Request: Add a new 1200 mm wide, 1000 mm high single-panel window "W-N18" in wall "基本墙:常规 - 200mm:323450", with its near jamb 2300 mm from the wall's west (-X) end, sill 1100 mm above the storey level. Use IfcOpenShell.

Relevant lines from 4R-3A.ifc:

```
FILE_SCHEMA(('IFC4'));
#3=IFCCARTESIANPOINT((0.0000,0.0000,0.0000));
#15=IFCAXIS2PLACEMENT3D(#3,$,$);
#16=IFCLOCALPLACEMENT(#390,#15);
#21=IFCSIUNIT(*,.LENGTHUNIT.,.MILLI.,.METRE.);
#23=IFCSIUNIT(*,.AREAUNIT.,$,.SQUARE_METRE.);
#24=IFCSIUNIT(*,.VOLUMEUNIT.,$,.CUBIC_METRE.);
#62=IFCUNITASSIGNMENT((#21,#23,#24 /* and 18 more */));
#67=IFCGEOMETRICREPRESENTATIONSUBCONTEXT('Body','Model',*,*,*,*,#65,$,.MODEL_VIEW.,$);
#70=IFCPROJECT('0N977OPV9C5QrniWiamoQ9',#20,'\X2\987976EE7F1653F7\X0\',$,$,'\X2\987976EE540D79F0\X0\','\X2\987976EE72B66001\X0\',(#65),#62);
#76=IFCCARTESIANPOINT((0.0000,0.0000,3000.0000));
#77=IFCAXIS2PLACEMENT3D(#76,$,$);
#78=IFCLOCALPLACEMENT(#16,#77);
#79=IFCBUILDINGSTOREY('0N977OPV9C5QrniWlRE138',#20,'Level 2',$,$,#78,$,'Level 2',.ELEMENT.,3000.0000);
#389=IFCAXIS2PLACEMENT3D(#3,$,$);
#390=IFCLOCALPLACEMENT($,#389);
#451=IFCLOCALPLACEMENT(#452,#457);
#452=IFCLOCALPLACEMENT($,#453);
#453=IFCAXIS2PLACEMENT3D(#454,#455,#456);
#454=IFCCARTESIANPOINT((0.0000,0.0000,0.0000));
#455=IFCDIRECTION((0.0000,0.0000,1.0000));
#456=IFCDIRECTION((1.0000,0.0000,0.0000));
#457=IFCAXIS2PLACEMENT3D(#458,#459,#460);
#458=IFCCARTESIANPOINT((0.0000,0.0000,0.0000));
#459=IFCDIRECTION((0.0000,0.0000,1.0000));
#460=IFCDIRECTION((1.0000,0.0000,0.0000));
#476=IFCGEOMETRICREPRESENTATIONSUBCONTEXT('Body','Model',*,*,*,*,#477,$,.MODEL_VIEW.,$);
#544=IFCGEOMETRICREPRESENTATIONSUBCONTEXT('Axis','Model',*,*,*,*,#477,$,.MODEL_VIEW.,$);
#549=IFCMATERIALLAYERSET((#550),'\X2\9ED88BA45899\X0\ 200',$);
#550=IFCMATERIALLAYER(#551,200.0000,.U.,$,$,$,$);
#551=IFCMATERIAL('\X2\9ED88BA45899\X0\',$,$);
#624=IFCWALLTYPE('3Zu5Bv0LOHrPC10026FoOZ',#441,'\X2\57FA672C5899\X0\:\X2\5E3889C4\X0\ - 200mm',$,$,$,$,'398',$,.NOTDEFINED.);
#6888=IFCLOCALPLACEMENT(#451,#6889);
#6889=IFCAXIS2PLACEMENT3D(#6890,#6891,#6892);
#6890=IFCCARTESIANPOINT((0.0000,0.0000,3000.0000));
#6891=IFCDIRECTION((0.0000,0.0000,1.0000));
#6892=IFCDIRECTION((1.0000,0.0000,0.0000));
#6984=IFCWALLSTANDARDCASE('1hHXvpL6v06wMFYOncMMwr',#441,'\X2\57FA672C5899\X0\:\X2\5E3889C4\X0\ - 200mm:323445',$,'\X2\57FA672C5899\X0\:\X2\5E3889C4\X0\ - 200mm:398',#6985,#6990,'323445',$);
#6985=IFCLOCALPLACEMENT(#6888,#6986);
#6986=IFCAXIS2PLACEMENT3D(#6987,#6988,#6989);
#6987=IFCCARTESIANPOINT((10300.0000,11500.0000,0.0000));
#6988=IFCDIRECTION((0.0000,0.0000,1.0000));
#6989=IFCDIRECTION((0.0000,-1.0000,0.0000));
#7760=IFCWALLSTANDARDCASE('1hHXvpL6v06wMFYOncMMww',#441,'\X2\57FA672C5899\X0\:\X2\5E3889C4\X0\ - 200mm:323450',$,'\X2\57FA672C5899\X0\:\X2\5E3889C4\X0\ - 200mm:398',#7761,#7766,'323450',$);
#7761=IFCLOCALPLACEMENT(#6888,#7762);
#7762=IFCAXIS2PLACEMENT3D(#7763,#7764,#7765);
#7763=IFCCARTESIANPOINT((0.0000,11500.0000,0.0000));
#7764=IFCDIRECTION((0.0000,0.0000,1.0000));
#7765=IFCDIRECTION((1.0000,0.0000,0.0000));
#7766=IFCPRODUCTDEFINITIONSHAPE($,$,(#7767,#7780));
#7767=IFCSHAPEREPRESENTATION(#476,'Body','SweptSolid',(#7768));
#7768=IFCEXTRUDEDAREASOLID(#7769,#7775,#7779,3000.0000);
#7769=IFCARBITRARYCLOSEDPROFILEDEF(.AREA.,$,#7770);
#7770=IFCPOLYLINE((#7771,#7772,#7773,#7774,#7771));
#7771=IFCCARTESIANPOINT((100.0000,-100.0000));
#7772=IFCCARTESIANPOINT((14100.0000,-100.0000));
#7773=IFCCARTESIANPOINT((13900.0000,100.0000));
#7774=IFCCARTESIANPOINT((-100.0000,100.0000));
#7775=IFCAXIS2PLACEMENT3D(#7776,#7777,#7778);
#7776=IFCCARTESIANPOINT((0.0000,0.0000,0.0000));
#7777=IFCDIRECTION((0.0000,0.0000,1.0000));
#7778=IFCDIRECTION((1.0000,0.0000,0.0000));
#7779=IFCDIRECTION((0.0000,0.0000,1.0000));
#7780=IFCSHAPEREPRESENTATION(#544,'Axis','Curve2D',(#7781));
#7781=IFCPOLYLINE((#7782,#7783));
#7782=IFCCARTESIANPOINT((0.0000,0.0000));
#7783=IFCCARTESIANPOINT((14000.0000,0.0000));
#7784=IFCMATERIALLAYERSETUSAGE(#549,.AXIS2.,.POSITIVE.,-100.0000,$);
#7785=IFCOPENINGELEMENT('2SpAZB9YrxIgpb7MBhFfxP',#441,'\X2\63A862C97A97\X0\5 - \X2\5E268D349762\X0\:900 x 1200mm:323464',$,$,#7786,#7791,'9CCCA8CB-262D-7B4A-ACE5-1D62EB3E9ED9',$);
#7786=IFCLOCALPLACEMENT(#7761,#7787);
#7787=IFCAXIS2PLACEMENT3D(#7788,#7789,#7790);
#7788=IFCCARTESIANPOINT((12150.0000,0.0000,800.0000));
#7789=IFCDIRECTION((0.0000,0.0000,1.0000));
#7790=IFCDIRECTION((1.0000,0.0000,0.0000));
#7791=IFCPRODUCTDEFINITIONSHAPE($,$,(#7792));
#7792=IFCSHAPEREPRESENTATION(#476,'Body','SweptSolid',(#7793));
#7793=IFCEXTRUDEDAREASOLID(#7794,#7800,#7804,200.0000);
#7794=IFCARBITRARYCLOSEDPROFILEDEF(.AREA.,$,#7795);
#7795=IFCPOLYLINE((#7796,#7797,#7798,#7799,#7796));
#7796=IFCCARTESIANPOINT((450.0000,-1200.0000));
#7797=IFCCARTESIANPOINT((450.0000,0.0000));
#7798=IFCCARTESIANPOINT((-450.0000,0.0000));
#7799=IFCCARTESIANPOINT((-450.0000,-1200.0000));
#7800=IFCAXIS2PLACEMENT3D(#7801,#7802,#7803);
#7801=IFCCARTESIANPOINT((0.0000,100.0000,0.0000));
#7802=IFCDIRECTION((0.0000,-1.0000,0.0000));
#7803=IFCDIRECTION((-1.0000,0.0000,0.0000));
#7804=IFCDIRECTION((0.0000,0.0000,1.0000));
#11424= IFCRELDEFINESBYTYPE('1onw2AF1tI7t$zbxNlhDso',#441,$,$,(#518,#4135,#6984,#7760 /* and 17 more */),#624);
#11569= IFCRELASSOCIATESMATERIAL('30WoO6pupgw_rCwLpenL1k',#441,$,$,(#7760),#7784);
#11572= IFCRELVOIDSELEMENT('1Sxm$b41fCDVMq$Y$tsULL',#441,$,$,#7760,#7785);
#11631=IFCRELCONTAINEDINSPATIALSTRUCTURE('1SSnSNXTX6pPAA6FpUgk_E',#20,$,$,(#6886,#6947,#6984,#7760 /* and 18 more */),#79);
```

```python
import numpy as np
import ifcopenshell
import ifcopenshell.api.feature
import ifcopenshell.api.geometry
import ifcopenshell.api.root
import ifcopenshell.api.spatial
import ifcopenshell.geom
import ifcopenshell.util.element
import ifcopenshell.util.placement
import ifcopenshell.util.representation
import ifcopenshell.util.shape
import ifcopenshell.util.unit

model = ifcopenshell.open("4R-3A.ifc")
unit_scale = ifcopenshell.util.unit.calculate_unit_scale(model)
settings = ifcopenshell.geom.settings()


def volume(element):
    """Net volume in cubic metres, openings subtracted."""
    shape = ifcopenshell.geom.create_shape(settings, element)
    return ifcopenshell.util.shape.get_volume(shape.geometry)


wall = model.by_id(7760)
storey = ifcopenshell.util.element.get_container(wall, ifc_class="IfcBuildingStorey")
context = ifcopenshell.util.representation.get_context(model, "Model", "Body", "MODEL_VIEW")
before = volume(wall)

width, height, from_end, sill = 1.2, 1, 2.3, 1.1  # metres

# The wall runs along its own X axis, and the end named is its -X end.
wall_shape = ifcopenshell.geom.create_shape(settings, wall)
x, y, z = ifcopenshell.util.shape.get_vertices(wall_shape.geometry).T
start = x.min() + from_end
face, thickness = float(y.min()), float(y.max() - y.min())
wall_matrix = ifcopenshell.util.placement.get_local_placement(wall.ObjectPlacement)
level = ifcopenshell.util.placement.get_local_placement(storey.ObjectPlacement)[2, 3]


def in_wall(x, y):
    """Placement at x, y metres in the wall's axes, at sill height."""
    matrix = wall_matrix.copy()
    matrix[:, 3] = wall_matrix @ np.array([x / unit_scale, y / unit_scale, 0.0, 1.0])
    matrix[2, 3] = level + sill / unit_scale
    return matrix


# Opening: a box that overshoots both wall faces by 50 mm.
opening = ifcopenshell.api.root.create_entity(model, ifc_class="IfcOpeningElement", predefined_type="OPENING")
box = ifcopenshell.api.geometry.add_wall_representation(
    model, context=context, length=width, height=height, thickness=thickness + 0.1
)
ifcopenshell.api.geometry.assign_representation(model, product=opening, representation=box)
ifcopenshell.api.geometry.edit_object_placement(model, product=opening, matrix=in_wall(start, face - 0.05), is_si=False)
ifcopenshell.api.feature.add_feature(model, feature=opening, element=wall)

window = ifcopenshell.api.root.create_entity(model, ifc_class="IfcWindow", name="W-N18", predefined_type="WINDOW")
window.OverallWidth, window.OverallHeight = width / unit_scale, height / unit_scale
window.PartitioningType = "SINGLE_PANEL"
body = ifcopenshell.api.geometry.add_window_representation(
    model,
    context=context,
    overall_width=window.OverallWidth,
    overall_height=window.OverallHeight,
    partition_type="SINGLE_PANEL",
)
ifcopenshell.api.geometry.assign_representation(model, product=window, representation=body)
ifcopenshell.api.spatial.assign_container(model, products=[window], relating_structure=storey)
ifcopenshell.api.feature.add_filling(model, opening=opening, element=window)

# Centre the window in the wall's thickness.
ifcopenshell.api.geometry.edit_object_placement(model, product=window, matrix=in_wall(start, face), is_si=False)
window_shape = ifcopenshell.geom.create_shape(settings, window)
depth = ifcopenshell.util.shape.get_vertices(window_shape.geometry)[:, 1]
offset = face + thickness / 2 - (depth.min() + depth.max()) / 2
ifcopenshell.api.geometry.edit_object_placement(model, product=window, matrix=in_wall(start, offset), is_si=False)

after = volume(wall)

print(f"wall volume {before:.3f} -> {after:.3f} m3")

model.write("4R-3A_edited.ifc")
```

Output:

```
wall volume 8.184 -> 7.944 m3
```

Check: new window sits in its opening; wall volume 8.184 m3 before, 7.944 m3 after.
